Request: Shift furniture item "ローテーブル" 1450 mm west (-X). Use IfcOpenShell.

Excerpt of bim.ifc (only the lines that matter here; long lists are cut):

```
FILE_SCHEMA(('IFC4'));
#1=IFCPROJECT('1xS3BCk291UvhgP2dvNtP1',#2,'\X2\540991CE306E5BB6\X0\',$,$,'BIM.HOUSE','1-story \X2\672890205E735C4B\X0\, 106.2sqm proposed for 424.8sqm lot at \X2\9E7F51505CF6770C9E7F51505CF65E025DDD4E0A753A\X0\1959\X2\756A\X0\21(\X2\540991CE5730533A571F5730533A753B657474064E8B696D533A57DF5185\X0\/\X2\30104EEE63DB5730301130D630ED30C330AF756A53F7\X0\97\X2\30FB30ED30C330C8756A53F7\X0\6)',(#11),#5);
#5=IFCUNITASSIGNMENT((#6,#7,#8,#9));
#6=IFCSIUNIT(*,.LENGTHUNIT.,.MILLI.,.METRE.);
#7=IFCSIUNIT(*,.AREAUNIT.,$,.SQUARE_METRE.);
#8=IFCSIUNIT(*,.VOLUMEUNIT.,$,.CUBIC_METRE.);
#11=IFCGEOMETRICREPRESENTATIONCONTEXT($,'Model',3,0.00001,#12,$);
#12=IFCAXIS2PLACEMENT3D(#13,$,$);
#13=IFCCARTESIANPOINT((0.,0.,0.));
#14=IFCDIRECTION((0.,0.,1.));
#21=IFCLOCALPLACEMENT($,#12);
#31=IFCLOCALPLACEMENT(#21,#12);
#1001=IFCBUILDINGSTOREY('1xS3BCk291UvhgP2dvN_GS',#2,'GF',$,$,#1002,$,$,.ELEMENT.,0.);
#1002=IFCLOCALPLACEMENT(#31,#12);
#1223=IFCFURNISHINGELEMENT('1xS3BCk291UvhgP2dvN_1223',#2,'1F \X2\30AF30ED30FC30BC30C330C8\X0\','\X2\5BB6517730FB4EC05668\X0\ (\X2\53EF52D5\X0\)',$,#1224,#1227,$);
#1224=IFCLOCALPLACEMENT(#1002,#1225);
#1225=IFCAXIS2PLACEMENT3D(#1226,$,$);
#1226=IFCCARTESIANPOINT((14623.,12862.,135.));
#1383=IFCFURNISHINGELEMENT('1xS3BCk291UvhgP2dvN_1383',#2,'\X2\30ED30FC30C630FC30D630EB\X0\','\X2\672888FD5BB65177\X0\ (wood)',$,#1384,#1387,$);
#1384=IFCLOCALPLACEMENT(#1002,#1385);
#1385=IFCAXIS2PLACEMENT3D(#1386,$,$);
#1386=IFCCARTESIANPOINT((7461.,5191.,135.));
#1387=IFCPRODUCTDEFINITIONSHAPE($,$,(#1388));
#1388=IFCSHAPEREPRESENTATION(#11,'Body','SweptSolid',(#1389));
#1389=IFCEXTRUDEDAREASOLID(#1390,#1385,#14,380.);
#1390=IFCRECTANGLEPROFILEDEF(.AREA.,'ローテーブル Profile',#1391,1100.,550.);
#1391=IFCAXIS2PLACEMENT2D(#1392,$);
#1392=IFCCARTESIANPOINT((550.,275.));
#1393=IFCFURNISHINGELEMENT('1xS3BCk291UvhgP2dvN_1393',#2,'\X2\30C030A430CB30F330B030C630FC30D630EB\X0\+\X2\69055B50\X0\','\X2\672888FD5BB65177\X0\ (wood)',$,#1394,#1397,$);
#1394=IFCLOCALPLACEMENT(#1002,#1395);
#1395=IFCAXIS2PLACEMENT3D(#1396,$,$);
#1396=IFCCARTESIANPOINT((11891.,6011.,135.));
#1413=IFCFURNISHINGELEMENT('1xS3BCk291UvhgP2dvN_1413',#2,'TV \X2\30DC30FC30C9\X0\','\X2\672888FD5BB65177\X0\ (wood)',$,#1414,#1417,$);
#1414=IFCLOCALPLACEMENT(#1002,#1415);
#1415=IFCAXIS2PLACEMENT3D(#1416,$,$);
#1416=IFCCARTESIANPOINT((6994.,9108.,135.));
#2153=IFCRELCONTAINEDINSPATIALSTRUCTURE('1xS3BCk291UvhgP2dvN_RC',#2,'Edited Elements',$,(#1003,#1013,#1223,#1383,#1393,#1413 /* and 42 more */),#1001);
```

```python
import ifcopenshell
import ifcopenshell.api.geometry
import ifcopenshell.util.placement
import ifcopenshell.util.unit

model = ifcopenshell.open("bim.ifc")
unit_scale = ifcopenshell.util.unit.calculate_unit_scale(model)

item = model.by_guid("1xS3BCk291UvhgP2dvN_1383")
matrix = ifcopenshell.util.placement.get_local_placement(item.ObjectPlacement)
matrix[0, 3] -= 1.45 / unit_scale
ifcopenshell.api.geometry.edit_object_placement(model, product=item, matrix=matrix, is_si=False)

print(ifcopenshell.util.placement.get_local_placement(item.ObjectPlacement).round(3) + 0.0)

model.write("bim_v2.ifc")
```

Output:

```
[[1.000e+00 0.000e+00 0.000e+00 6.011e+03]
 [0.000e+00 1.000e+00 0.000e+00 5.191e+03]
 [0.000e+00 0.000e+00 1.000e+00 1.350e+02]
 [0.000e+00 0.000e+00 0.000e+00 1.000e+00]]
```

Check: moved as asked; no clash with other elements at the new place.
